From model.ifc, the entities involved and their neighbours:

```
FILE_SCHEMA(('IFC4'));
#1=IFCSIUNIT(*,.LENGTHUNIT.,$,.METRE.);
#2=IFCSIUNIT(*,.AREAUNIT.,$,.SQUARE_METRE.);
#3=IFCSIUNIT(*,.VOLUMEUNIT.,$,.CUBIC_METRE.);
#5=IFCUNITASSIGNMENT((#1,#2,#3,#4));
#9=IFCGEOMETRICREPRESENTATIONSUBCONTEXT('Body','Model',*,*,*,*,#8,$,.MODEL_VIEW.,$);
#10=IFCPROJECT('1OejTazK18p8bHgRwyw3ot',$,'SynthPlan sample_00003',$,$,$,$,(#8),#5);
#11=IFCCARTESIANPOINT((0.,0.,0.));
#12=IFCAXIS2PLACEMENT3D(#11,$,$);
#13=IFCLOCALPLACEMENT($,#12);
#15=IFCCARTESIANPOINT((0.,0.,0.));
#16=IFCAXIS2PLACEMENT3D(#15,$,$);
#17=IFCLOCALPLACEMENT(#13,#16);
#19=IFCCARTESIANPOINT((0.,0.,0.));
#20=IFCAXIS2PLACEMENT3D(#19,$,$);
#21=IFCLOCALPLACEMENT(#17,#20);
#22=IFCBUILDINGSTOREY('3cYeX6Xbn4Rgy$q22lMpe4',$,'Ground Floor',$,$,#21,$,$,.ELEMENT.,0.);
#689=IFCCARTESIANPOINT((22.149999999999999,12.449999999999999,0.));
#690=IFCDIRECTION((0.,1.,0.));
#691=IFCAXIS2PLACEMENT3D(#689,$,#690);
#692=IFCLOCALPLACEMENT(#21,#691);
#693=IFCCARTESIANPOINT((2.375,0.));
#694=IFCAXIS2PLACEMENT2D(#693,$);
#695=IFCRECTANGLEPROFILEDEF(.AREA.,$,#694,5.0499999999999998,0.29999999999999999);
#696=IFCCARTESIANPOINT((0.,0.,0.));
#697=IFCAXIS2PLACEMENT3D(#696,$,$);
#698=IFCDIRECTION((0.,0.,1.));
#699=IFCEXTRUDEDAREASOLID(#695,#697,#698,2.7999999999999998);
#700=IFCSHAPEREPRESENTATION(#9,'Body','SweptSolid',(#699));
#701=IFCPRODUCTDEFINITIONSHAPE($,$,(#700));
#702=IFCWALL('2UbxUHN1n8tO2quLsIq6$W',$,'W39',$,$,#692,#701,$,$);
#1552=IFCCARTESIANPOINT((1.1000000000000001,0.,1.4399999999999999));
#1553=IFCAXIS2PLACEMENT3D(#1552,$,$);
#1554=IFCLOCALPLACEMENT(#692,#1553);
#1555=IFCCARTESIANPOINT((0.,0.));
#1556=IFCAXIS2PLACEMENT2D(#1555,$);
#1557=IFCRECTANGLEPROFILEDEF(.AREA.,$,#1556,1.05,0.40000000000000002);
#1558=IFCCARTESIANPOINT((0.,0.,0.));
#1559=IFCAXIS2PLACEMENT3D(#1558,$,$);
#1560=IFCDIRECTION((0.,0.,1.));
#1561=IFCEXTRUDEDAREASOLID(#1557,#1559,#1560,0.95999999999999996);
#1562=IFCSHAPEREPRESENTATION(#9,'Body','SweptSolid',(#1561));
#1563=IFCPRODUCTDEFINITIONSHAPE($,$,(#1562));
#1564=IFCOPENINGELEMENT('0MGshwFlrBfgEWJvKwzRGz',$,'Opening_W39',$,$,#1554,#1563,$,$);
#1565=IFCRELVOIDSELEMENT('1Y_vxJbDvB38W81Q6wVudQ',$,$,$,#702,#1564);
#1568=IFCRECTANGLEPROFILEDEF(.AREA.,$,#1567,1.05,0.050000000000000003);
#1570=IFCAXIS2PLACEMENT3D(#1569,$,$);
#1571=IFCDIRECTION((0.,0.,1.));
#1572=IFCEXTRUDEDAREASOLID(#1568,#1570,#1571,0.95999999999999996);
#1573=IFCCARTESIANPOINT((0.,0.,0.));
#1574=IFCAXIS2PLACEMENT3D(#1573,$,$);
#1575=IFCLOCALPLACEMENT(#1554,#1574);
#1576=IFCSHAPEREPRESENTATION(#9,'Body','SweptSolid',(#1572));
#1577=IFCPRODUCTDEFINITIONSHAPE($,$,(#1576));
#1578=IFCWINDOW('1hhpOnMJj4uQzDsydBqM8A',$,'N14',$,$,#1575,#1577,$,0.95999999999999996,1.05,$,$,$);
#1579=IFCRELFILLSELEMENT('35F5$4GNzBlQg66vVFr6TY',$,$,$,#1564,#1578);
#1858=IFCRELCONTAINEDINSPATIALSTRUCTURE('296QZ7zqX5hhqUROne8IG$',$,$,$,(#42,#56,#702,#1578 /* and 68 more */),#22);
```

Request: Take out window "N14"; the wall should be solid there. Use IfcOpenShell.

```python
import ifcopenshell
import ifcopenshell.api.feature
import ifcopenshell.api.root
import ifcopenshell.geom
import ifcopenshell.util.shape

model = ifcopenshell.open("model.ifc")
settings = ifcopenshell.geom.settings()


def volume(element):
    """Net volume in cubic metres, openings subtracted."""
    shape = ifcopenshell.geom.create_shape(settings, element)
    return ifcopenshell.util.shape.get_volume(shape.geometry)


window = model.by_guid("1hhpOnMJj4uQzDsydBqM8A")
opening = window.FillsVoids[0].RelatingOpeningElement
wall = opening.VoidsElements[0].RelatingBuildingElement
before = volume(wall)

ifcopenshell.api.root.remove_product(model, product=window)
ifcopenshell.api.feature.remove_feature(model, feature=opening)

after = volume(wall)

print(f"wall volume {before:.3f} -> {after:.3f} m3")

model.write("model_v2.ifc")
```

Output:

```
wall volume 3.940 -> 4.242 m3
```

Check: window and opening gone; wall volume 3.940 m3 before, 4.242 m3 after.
